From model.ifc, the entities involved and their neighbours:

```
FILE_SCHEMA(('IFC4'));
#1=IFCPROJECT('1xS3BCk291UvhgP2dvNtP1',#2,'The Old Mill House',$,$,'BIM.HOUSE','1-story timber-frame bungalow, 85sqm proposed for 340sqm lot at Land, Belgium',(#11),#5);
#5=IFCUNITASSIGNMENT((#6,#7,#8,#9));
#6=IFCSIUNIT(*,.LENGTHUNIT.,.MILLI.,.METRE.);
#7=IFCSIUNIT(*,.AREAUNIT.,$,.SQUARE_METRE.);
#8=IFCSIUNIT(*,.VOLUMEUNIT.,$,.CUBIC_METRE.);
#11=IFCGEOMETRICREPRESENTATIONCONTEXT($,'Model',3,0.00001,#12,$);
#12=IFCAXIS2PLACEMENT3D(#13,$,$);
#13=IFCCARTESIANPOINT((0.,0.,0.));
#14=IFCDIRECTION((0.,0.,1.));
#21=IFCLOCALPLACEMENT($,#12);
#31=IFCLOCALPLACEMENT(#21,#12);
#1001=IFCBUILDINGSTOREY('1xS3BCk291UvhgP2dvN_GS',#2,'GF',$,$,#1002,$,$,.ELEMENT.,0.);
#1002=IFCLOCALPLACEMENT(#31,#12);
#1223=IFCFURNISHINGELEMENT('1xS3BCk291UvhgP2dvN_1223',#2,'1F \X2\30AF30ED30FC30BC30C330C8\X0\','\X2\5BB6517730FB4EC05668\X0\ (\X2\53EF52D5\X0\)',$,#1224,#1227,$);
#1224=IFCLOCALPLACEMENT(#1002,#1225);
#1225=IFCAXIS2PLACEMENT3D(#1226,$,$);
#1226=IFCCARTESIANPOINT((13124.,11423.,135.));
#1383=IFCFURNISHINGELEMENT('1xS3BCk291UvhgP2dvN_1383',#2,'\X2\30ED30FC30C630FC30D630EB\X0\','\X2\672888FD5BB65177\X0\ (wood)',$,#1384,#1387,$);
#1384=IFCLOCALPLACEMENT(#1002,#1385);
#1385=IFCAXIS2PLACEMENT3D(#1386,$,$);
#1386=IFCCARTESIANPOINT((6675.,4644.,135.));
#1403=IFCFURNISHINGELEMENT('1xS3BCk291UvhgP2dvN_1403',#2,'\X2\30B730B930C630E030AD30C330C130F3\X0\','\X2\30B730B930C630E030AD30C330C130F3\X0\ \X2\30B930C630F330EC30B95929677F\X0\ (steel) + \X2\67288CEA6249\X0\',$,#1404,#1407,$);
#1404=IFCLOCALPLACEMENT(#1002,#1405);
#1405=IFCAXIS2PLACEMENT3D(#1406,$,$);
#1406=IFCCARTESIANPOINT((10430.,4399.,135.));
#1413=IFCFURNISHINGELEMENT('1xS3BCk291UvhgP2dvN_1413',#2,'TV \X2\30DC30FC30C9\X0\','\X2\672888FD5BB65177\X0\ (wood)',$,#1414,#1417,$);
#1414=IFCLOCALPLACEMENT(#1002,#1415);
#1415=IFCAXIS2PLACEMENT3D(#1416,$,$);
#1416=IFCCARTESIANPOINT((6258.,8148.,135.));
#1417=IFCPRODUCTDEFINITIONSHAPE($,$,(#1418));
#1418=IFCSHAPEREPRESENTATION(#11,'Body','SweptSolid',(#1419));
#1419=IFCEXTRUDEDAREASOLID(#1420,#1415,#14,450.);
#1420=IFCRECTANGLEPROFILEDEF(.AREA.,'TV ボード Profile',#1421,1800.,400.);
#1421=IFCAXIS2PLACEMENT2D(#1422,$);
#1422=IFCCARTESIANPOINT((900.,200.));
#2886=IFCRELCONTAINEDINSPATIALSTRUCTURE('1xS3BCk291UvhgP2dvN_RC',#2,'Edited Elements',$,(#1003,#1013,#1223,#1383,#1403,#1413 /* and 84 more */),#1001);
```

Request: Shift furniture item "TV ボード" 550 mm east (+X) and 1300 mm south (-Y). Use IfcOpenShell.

```python
import ifcopenshell
import ifcopenshell.api.geometry
import ifcopenshell.util.placement
import ifcopenshell.util.unit

model = ifcopenshell.open("model.ifc")
unit_scale = ifcopenshell.util.unit.calculate_unit_scale(model)

item = model.by_id(1413)
matrix = ifcopenshell.util.placement.get_local_placement(item.ObjectPlacement)
matrix[0, 3] += 0.55 / unit_scale
matrix[1, 3] -= 1.3 / unit_scale
ifcopenshell.api.geometry.edit_object_placement(model, product=item, matrix=matrix, is_si=False)

print(ifcopenshell.util.placement.get_local_placement(item.ObjectPlacement).round(3) + 0.0)

model.write("model-out.ifc")
```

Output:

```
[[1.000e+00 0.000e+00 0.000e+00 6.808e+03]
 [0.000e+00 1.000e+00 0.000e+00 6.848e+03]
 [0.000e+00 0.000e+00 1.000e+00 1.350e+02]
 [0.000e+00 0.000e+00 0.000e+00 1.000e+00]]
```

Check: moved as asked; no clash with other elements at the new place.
